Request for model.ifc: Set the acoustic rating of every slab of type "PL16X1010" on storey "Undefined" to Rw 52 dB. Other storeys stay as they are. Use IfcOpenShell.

First a look at what the model holds.

```python
import ifcopenshell
import ifcopenshell.util.element

model = ifcopenshell.open("model.ifc")
print(model.schema)
storey = next(s for s in model.by_type("IfcBuildingStorey") if s.Name == "Undefined")
slabs = [e for e in ifcopenshell.util.element.get_decomposition(storey) if e.is_a("IfcSlab")]
seen = {}
for e in slabs:
    element_type = ifcopenshell.util.element.get_type(e)
    key = (element_type.Name if element_type != e and element_type else None, ifcopenshell.util.element.get_pset(e, "Pset_SlabCommon", "AcousticRating"))
    seen[key] = seen.get(key, 0) + 1
for (name, value), count in sorted(seen.items(), key=str):
    print(count, "x", name, "|", value)
```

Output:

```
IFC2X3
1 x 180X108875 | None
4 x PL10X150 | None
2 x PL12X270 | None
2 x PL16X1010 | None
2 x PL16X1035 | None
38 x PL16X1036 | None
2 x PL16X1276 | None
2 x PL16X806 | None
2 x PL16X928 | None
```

```python
import ifcopenshell
import ifcopenshell.api.pset
import ifcopenshell.util.element

model = ifcopenshell.open("model.ifc")

storey = next(s for s in model.by_type("IfcBuildingStorey") if s.Name == "Undefined")
slabs = [e for e in ifcopenshell.util.element.get_decomposition(storey) if e.is_a("IfcSlab")]

count = 0
for e in slabs:
    element_type = ifcopenshell.util.element.get_type(e)
    if element_type in (None, e) or element_type.Name != "PL16X1010":
        continue
    # add_pset returns the element's existing set when there is one.
    pset = ifcopenshell.api.pset.add_pset(model, product=e, name="Pset_SlabCommon")
    ifcopenshell.api.pset.edit_pset(model, pset=pset, properties={"AcousticRating": "Rw 52 dB"})
    count += 1

print(count, "slabs updated")

model.write("model_rev.ifc")
```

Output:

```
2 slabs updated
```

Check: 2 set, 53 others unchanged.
